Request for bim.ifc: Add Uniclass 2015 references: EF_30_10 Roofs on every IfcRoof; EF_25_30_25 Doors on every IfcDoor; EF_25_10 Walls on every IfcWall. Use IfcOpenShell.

First a look at what the model holds.

```python
import ifcopenshell

model = ifcopenshell.open("bim.ifc")
print(model.schema)
print("classifications:", [c.Name for c in model.by_type("IfcClassification")])
for ifc_class in ("IfcDoor", "IfcRoof", "IfcStair", "IfcWall", "IfcWindow"):
    print(ifc_class, len(model.by_type(ifc_class)))
```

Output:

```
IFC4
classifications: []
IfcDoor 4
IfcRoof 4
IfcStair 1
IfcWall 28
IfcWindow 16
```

```python
import ifcopenshell
import ifcopenshell.api.classification

model = ifcopenshell.open("bim.ifc")

system = ifcopenshell.api.classification.add_classification(model, classification="Uniclass 2015")

codes = {
    "IfcRoof": ("EF_30_10", "Roofs"),
    "IfcDoor": ("EF_25_30_25", "Doors"),
    "IfcWall": ("EF_25_10", "Walls"),
}
for ifc_class, (code, name) in codes.items():
    products = model.by_type(ifc_class)
    ifcopenshell.api.classification.add_reference(
        model, products=products, classification=system, identification=code, name=name
    )
    print(code, len(products))

model.write("bim_updated.ifc")
```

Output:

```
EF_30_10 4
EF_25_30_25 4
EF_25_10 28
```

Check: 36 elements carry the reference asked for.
